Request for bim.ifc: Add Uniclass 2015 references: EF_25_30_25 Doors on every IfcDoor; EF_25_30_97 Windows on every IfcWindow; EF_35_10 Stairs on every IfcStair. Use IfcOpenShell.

First a look at what the model holds.

```python
import ifcopenshell

model = ifcopenshell.open("bim.ifc")
print(model.schema)
print("classifications:", [c.Name for c in model.by_type("IfcClassification")])
for ifc_class in ("IfcDoor", "IfcRoof", "IfcStair", "IfcWall", "IfcWindow"):
    print(ifc_class, len(model.by_type(ifc_class)))
```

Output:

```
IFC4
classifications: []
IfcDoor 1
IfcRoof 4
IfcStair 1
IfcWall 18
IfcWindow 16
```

```python
import ifcopenshell
import ifcopenshell.api.classification

model = ifcopenshell.open("bim.ifc")

system = ifcopenshell.api.classification.add_classification(model, classification="Uniclass 2015")

codes = {
    "IfcDoor": ("EF_25_30_25", "Doors"),
    "IfcWindow": ("EF_25_30_97", "Windows"),
    "IfcStair": ("EF_35_10", "Stairs"),
}
for ifc_class, (code, name) in codes.items():
    products = model.by_type(ifc_class)
    ifcopenshell.api.classification.add_reference(
        model, products=products, classification=system, identification=code, name=name
    )
    print(code, len(products))

model.write("bim-out.ifc")
```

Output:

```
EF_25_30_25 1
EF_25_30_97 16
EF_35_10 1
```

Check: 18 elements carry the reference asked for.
